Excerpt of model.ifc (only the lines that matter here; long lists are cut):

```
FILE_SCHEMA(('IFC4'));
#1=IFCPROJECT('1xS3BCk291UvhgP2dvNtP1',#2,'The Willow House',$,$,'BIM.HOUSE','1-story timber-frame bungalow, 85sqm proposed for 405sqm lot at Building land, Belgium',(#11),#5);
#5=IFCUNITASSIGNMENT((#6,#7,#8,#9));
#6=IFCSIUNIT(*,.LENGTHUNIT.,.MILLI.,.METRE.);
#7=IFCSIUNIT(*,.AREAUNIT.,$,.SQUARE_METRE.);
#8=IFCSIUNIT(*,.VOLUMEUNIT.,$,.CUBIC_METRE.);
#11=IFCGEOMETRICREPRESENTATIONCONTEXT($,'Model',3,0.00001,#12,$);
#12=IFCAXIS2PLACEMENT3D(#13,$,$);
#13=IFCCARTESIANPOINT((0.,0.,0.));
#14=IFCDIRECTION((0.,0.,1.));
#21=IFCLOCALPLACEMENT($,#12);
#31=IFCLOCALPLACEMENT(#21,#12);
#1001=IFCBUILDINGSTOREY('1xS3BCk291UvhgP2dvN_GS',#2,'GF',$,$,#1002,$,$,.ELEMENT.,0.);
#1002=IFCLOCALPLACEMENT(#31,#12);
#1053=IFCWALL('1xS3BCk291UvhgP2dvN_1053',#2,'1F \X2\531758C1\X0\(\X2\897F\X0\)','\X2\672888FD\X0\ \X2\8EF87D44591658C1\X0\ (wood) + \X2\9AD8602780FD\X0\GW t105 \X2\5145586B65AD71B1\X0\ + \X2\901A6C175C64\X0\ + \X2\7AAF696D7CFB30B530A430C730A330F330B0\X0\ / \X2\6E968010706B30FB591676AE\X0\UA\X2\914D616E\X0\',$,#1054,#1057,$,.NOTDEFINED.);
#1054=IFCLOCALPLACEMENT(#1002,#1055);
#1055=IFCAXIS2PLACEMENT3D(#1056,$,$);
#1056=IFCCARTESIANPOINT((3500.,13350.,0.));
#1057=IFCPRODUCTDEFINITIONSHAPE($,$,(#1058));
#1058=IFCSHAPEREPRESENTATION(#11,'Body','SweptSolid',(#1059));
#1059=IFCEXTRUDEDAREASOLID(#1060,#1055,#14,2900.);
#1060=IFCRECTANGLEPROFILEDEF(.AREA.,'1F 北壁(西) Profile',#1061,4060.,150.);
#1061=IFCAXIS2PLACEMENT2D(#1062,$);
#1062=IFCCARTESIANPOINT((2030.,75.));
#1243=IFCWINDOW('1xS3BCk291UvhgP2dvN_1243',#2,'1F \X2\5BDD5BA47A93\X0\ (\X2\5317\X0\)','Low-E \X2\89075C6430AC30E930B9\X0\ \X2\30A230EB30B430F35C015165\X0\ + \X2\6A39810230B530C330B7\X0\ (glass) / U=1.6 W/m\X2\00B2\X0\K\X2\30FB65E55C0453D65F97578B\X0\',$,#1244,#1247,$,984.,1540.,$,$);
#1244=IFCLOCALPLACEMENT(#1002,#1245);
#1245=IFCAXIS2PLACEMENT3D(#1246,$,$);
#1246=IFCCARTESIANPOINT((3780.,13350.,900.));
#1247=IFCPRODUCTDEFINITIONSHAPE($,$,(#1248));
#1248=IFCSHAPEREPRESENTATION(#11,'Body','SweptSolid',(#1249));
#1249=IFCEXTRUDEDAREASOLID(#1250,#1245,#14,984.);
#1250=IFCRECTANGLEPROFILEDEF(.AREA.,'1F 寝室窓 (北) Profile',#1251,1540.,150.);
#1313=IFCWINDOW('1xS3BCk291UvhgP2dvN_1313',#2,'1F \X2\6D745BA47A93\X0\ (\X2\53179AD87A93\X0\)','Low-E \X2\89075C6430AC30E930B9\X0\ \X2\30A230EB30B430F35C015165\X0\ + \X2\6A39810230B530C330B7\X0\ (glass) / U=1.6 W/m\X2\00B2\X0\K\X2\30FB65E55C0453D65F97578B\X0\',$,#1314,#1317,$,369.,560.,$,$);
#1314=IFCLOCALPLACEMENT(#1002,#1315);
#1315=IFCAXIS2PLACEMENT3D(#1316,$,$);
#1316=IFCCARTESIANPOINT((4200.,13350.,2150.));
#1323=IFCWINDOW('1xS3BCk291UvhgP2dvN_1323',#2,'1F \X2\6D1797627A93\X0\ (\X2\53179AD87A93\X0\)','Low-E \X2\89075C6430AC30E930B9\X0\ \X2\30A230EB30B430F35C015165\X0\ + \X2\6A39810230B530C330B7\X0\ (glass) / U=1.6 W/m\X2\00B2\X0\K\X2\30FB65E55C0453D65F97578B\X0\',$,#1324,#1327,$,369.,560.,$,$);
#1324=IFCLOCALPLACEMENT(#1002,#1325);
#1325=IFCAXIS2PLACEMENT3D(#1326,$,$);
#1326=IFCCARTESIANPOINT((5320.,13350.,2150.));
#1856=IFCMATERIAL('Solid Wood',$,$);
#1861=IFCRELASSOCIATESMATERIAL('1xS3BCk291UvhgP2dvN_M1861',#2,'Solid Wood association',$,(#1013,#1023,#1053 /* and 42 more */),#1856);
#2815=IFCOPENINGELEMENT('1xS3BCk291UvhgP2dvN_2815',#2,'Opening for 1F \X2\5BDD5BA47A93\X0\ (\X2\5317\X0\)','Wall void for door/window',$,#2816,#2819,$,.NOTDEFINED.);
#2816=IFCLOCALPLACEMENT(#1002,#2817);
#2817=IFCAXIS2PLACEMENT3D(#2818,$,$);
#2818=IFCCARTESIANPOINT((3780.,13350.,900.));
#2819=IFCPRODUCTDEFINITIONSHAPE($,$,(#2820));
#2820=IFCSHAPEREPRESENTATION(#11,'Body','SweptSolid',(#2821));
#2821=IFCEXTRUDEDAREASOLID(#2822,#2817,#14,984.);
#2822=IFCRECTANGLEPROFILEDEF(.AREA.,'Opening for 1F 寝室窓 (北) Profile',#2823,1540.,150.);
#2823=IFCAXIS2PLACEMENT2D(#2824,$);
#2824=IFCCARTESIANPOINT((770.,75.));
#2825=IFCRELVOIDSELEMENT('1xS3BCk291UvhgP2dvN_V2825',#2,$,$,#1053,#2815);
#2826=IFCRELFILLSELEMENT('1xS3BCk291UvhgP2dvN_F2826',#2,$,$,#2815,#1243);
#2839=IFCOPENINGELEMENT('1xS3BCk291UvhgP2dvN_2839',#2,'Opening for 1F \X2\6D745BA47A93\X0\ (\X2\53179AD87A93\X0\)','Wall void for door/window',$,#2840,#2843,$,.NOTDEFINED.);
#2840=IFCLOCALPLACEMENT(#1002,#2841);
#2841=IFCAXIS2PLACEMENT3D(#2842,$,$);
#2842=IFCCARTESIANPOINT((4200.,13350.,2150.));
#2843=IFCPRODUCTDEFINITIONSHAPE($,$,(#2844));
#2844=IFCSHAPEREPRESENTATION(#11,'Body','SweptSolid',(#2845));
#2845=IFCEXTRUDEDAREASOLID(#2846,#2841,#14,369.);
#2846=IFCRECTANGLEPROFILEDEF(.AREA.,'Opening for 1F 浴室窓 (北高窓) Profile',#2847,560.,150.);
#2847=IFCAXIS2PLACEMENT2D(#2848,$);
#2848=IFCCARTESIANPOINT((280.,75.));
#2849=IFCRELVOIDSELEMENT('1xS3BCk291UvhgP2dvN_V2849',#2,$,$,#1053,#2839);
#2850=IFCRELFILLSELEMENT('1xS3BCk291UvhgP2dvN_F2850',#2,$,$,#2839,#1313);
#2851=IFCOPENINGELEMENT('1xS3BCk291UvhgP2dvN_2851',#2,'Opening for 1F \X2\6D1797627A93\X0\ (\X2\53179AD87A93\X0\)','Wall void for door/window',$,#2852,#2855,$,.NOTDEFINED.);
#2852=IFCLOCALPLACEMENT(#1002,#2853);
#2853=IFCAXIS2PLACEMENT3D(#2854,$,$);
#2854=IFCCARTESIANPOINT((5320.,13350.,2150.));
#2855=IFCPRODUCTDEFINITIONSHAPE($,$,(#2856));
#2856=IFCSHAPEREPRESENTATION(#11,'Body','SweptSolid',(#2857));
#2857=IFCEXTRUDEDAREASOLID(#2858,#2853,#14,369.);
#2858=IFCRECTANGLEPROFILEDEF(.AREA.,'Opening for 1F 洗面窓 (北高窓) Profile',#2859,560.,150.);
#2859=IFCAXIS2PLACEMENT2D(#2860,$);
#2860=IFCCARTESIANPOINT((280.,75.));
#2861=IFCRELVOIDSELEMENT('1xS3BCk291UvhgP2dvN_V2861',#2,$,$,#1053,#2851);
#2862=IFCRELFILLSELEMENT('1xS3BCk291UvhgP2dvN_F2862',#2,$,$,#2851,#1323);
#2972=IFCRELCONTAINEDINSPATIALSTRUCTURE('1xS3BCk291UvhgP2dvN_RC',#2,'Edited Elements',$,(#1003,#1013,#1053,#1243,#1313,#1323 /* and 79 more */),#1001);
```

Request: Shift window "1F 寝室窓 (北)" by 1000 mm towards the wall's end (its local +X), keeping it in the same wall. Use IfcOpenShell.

```python
import ifcopenshell
import ifcopenshell.api.geometry
import ifcopenshell.util.placement
import ifcopenshell.util.unit

model = ifcopenshell.open("model.ifc")
unit_scale = ifcopenshell.util.unit.calculate_unit_scale(model)

window = model.by_guid("1xS3BCk291UvhgP2dvN_1243")
opening = window.FillsVoids[0].RelatingOpeningElement
wall = opening.VoidsElements[0].RelatingBuildingElement

wall_matrix = ifcopenshell.util.placement.get_local_placement(wall.ObjectPlacement)
shift = wall_matrix[:3, 0] * 1 / unit_scale
before = ifcopenshell.util.placement.get_local_placement(window.ObjectPlacement)[:3, 3].copy()

# The window is not placed relative to its opening, so move both.
for product in (opening, window):
    matrix = ifcopenshell.util.placement.get_local_placement(product.ObjectPlacement)
    matrix[:3, 3] += shift
    ifcopenshell.api.geometry.edit_object_placement(model, product=product, matrix=matrix, is_si=False)

after = ifcopenshell.util.placement.get_local_placement(window.ObjectPlacement)[:3, 3]
print("window moved by", (after - before).round(3) + 0.0)

model.write("model_edited.ifc")
```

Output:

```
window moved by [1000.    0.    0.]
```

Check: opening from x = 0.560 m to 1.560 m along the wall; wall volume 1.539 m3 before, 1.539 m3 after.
